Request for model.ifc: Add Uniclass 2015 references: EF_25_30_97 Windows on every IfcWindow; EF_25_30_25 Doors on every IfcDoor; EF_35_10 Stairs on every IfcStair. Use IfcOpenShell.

First a look at what the model holds.

```python
import ifcopenshell

model = ifcopenshell.open("model.ifc")
print(model.schema)
print("classifications:", [c.Name for c in model.by_type("IfcClassification")])
for ifc_class in ("IfcDoor", "IfcRoof", "IfcStair", "IfcWall", "IfcWindow"):
    print(ifc_class, len(model.by_type(ifc_class)))
```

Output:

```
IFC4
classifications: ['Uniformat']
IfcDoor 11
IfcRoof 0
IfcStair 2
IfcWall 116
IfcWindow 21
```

```python
import ifcopenshell
import ifcopenshell.api.classification

model = ifcopenshell.open("model.ifc")

system = ifcopenshell.api.classification.add_classification(model, classification="Uniclass 2015")

codes = {
    "IfcWindow": ("EF_25_30_97", "Windows"),
    "IfcDoor": ("EF_25_30_25", "Doors"),
    "IfcStair": ("EF_35_10", "Stairs"),
}
for ifc_class, (code, name) in codes.items():
    products = model.by_type(ifc_class)
    ifcopenshell.api.classification.add_reference(
        model, products=products, classification=system, identification=code, name=name
    )
    print(code, len(products))

model.write("model_v2.ifc")
```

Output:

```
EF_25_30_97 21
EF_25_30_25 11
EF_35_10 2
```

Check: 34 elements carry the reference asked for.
